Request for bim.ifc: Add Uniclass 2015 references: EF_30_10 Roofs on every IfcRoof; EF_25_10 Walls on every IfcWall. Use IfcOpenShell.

First a look at what the model holds.

```python
import ifcopenshell

model = ifcopenshell.open("bim.ifc")
print(model.schema)
print("classifications:", [c.Name for c in model.by_type("IfcClassification")])
for ifc_class in ("IfcDoor", "IfcRoof", "IfcStair", "IfcWall", "IfcWindow"):
    print(ifc_class, len(model.by_type(ifc_class)))
```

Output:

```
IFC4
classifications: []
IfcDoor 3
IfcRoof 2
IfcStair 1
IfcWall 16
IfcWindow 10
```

```python
import ifcopenshell
import ifcopenshell.api.classification

model = ifcopenshell.open("bim.ifc")

system = ifcopenshell.api.classification.add_classification(model, classification="Uniclass 2015")

codes = {
    "IfcRoof": ("EF_30_10", "Roofs"),
    "IfcWall": ("EF_25_10", "Walls"),
}
for ifc_class, (code, name) in codes.items():
    products = model.by_type(ifc_class)
    ifcopenshell.api.classification.add_reference(
        model, products=products, classification=system, identification=code, name=name
    )
    print(code, len(products))

model.write("bim_v2.ifc")
```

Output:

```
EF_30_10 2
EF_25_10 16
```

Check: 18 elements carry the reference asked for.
